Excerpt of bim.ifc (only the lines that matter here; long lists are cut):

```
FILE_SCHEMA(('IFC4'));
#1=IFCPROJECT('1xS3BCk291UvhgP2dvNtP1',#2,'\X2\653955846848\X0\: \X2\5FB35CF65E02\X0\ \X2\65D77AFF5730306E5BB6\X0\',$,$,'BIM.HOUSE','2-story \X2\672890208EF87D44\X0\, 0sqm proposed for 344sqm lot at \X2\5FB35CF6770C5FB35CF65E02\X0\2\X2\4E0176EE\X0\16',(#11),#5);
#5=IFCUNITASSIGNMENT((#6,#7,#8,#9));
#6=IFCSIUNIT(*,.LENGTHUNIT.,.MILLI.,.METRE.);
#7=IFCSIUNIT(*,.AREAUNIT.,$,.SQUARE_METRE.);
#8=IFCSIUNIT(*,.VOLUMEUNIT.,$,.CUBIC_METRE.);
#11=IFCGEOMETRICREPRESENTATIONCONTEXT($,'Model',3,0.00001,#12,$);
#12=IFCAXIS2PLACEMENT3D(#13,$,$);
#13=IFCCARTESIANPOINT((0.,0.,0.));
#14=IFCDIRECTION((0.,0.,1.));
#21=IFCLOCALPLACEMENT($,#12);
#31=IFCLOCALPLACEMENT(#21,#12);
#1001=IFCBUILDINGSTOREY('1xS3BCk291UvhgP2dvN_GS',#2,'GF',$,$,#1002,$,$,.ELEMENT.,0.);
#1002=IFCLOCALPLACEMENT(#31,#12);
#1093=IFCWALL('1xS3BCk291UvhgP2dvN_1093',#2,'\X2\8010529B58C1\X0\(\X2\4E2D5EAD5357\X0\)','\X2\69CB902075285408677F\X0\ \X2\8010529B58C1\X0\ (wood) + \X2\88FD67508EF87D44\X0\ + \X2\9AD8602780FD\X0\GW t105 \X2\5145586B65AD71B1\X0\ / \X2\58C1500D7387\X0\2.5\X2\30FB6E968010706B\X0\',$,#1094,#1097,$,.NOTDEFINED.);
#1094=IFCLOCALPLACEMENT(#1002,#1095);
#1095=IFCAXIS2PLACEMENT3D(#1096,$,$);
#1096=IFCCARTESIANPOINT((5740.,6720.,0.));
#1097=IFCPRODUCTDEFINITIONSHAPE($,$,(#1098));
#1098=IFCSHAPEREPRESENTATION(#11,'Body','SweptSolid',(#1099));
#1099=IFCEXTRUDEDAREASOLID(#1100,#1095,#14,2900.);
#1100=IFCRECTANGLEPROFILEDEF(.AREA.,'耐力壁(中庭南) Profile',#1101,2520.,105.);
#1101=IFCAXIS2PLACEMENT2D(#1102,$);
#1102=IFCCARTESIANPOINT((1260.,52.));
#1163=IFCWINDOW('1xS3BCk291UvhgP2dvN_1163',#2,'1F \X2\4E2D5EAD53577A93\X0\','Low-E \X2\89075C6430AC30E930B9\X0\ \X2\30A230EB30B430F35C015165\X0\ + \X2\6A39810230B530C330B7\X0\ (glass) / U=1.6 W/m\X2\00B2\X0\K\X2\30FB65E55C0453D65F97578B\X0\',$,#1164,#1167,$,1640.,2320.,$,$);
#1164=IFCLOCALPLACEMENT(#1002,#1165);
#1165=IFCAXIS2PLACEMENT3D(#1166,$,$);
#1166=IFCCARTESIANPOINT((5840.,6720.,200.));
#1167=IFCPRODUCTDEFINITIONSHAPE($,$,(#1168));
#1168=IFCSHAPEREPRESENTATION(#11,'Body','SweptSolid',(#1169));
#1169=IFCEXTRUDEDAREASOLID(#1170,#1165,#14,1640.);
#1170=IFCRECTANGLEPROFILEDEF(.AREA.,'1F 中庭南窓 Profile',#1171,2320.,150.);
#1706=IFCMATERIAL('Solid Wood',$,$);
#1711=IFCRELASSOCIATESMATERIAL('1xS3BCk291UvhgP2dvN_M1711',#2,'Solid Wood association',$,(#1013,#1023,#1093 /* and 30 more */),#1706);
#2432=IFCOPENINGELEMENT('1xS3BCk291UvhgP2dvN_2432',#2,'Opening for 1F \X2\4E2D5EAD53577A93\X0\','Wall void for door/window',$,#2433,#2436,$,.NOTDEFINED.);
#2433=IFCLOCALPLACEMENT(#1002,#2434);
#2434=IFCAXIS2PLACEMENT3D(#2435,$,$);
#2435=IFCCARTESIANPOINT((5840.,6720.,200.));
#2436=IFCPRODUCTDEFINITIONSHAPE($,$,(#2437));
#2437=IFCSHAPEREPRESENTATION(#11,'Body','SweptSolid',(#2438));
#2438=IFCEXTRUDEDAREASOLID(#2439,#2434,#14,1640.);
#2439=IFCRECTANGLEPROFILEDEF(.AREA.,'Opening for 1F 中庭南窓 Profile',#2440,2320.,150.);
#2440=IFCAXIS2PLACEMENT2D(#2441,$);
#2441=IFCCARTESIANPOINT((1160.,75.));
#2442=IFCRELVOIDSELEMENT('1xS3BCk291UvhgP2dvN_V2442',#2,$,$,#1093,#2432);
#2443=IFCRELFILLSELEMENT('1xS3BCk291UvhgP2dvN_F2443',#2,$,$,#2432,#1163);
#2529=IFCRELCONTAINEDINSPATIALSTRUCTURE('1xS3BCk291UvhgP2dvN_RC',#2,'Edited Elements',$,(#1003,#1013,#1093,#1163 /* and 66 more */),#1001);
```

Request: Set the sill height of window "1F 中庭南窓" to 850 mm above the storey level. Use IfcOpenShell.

```python
import numpy as np
import ifcopenshell
import ifcopenshell.api.geometry
import ifcopenshell.geom
import ifcopenshell.util.element
import ifcopenshell.util.placement
import ifcopenshell.util.shape
import ifcopenshell.util.unit

model = ifcopenshell.open("bim.ifc")
unit_scale = ifcopenshell.util.unit.calculate_unit_scale(model)

window = model.by_guid("1xS3BCk291UvhgP2dvN_1163")
opening = window.FillsVoids[0].RelatingOpeningElement
storey = ifcopenshell.util.element.get_container(window, ifc_class="IfcBuildingStorey")
level = ifcopenshell.util.placement.get_local_placement(storey.ObjectPlacement)[2, 3]

# The opening's origin need not be at the sill, so measure its lowest point.
shape = ifcopenshell.geom.create_shape(ifcopenshell.geom.settings(), opening)
bottom = ifcopenshell.util.shape.get_shape_bottom_elevation(shape, shape.geometry) / unit_scale
dz = level + 0.85 / unit_scale - bottom

shift = np.array([0.0, 0.0, dz])
# The window is not placed relative to its opening, so move both.
for product in (opening, window):
    matrix = ifcopenshell.util.placement.get_local_placement(product.ObjectPlacement)
    matrix[:3, 3] += shift
    ifcopenshell.api.geometry.edit_object_placement(model, product=product, matrix=matrix, is_si=False)

print(f"moved by {dz * unit_scale:+.3f} m")

model.write("bim_v2.ifc")
```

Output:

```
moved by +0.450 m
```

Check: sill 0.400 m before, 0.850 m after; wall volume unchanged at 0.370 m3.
